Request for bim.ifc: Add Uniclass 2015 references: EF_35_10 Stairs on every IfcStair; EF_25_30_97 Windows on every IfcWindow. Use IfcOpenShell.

First a look at what the model holds.

```python
import ifcopenshell

model = ifcopenshell.open("bim.ifc")
print(model.schema)
print("classifications:", [c.Name for c in model.by_type("IfcClassification")])
for ifc_class in ("IfcDoor", "IfcRoof", "IfcStair", "IfcWall", "IfcWindow"):
    print(ifc_class, len(model.by_type(ifc_class)))
```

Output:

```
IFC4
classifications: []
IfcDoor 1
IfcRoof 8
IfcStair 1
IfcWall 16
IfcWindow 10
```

```python
import ifcopenshell
import ifcopenshell.api.classification

model = ifcopenshell.open("bim.ifc")

system = ifcopenshell.api.classification.add_classification(model, classification="Uniclass 2015")

codes = {
    "IfcStair": ("EF_35_10", "Stairs"),
    "IfcWindow": ("EF_25_30_97", "Windows"),
}
for ifc_class, (code, name) in codes.items():
    products = model.by_type(ifc_class)
    ifcopenshell.api.classification.add_reference(
        model, products=products, classification=system, identification=code, name=name
    )
    print(code, len(products))

model.write("bim-out.ifc")
```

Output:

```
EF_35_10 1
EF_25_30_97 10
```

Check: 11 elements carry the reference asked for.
